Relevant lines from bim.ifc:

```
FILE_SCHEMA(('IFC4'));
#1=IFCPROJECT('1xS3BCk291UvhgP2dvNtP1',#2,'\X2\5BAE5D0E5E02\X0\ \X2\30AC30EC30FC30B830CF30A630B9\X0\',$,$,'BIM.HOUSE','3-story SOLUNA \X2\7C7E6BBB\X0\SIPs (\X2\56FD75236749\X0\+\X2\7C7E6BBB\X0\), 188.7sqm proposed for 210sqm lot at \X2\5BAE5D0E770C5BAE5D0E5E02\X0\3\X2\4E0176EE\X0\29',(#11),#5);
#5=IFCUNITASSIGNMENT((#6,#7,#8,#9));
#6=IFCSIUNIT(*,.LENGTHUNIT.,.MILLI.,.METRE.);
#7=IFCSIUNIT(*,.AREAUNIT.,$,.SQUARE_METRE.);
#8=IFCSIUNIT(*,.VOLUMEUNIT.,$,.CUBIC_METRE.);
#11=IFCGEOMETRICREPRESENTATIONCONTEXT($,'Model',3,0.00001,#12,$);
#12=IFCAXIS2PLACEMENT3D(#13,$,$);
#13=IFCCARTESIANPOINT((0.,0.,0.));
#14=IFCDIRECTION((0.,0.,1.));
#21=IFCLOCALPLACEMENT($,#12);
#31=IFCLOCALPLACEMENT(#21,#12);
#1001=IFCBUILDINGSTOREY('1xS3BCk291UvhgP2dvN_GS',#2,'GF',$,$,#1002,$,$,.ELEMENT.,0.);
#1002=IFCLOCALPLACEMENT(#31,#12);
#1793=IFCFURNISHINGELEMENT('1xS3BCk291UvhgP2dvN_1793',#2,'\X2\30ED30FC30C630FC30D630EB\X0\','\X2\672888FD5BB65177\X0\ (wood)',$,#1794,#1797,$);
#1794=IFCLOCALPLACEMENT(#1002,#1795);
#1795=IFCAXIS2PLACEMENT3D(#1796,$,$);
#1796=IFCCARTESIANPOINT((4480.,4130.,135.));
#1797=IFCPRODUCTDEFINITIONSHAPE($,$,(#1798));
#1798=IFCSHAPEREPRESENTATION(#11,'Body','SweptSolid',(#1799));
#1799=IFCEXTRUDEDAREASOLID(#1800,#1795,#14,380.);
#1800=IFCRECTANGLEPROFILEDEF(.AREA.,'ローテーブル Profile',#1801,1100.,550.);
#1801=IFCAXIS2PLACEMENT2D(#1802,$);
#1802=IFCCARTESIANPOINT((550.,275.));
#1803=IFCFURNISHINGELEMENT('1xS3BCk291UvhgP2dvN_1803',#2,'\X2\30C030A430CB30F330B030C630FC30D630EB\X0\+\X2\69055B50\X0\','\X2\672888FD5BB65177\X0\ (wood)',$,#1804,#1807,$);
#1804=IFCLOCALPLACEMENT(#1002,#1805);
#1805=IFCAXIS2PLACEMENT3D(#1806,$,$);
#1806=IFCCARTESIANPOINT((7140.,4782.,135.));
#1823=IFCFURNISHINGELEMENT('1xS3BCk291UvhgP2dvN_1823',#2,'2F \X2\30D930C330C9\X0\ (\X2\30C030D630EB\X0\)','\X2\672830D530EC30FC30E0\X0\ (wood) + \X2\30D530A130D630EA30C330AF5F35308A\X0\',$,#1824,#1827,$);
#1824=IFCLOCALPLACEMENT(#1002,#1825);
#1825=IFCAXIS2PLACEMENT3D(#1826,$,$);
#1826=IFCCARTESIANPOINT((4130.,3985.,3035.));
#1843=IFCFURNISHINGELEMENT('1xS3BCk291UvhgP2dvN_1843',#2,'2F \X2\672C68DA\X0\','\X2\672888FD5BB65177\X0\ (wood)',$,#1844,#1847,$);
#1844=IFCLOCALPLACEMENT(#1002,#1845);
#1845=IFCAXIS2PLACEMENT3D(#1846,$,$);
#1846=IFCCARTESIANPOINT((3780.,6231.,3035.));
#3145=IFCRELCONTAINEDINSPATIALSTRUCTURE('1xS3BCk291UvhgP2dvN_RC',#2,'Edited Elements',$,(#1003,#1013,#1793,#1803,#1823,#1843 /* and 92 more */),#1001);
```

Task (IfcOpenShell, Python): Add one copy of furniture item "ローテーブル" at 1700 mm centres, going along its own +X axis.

```python
import ifcopenshell
import ifcopenshell.api.geometry
import ifcopenshell.api.root
import ifcopenshell.util.element
import ifcopenshell.util.placement
import ifcopenshell.util.unit

model = ifcopenshell.open("bim.ifc")
unit_scale = ifcopenshell.util.unit.calculate_unit_scale(model)


def reuse_history(source, copy):
    """copy_class also copies each property set's owner history, people and application; keep the originals."""
    for rel in copy.IsDefinedBy:
        if rel.is_a("IfcRelDefinesByProperties") and (history := rel.RelatingPropertyDefinition.OwnerHistory):
            rel.RelatingPropertyDefinition.OwnerHistory = source.OwnerHistory
            ifcopenshell.util.element.remove_deep2(model, history)


source = model.by_guid("1xS3BCk291UvhgP2dvN_1793")
base = ifcopenshell.util.placement.get_local_placement(source.ObjectPlacement)
step = base[:3, 0] * 1.7 / unit_scale

for i in range(1, 2):
    copy = ifcopenshell.api.root.copy_class(model, product=source)
    copy.Representation = ifcopenshell.util.element.copy_deep(
        model, source.Representation, exclude=["IfcGeometricRepresentationContext", "IfcRepresentationMap"]
    )
    reuse_history(source, copy)
    matrix = base.copy()
    matrix[:3, 3] += i * step
    print("added at", matrix[:3, 3].round(3) + 0.0)
    ifcopenshell.api.geometry.edit_object_placement(model, product=copy, matrix=matrix, is_si=False)

model.write("bim_updated.ifc")
```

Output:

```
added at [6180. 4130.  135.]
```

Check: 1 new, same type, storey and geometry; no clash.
